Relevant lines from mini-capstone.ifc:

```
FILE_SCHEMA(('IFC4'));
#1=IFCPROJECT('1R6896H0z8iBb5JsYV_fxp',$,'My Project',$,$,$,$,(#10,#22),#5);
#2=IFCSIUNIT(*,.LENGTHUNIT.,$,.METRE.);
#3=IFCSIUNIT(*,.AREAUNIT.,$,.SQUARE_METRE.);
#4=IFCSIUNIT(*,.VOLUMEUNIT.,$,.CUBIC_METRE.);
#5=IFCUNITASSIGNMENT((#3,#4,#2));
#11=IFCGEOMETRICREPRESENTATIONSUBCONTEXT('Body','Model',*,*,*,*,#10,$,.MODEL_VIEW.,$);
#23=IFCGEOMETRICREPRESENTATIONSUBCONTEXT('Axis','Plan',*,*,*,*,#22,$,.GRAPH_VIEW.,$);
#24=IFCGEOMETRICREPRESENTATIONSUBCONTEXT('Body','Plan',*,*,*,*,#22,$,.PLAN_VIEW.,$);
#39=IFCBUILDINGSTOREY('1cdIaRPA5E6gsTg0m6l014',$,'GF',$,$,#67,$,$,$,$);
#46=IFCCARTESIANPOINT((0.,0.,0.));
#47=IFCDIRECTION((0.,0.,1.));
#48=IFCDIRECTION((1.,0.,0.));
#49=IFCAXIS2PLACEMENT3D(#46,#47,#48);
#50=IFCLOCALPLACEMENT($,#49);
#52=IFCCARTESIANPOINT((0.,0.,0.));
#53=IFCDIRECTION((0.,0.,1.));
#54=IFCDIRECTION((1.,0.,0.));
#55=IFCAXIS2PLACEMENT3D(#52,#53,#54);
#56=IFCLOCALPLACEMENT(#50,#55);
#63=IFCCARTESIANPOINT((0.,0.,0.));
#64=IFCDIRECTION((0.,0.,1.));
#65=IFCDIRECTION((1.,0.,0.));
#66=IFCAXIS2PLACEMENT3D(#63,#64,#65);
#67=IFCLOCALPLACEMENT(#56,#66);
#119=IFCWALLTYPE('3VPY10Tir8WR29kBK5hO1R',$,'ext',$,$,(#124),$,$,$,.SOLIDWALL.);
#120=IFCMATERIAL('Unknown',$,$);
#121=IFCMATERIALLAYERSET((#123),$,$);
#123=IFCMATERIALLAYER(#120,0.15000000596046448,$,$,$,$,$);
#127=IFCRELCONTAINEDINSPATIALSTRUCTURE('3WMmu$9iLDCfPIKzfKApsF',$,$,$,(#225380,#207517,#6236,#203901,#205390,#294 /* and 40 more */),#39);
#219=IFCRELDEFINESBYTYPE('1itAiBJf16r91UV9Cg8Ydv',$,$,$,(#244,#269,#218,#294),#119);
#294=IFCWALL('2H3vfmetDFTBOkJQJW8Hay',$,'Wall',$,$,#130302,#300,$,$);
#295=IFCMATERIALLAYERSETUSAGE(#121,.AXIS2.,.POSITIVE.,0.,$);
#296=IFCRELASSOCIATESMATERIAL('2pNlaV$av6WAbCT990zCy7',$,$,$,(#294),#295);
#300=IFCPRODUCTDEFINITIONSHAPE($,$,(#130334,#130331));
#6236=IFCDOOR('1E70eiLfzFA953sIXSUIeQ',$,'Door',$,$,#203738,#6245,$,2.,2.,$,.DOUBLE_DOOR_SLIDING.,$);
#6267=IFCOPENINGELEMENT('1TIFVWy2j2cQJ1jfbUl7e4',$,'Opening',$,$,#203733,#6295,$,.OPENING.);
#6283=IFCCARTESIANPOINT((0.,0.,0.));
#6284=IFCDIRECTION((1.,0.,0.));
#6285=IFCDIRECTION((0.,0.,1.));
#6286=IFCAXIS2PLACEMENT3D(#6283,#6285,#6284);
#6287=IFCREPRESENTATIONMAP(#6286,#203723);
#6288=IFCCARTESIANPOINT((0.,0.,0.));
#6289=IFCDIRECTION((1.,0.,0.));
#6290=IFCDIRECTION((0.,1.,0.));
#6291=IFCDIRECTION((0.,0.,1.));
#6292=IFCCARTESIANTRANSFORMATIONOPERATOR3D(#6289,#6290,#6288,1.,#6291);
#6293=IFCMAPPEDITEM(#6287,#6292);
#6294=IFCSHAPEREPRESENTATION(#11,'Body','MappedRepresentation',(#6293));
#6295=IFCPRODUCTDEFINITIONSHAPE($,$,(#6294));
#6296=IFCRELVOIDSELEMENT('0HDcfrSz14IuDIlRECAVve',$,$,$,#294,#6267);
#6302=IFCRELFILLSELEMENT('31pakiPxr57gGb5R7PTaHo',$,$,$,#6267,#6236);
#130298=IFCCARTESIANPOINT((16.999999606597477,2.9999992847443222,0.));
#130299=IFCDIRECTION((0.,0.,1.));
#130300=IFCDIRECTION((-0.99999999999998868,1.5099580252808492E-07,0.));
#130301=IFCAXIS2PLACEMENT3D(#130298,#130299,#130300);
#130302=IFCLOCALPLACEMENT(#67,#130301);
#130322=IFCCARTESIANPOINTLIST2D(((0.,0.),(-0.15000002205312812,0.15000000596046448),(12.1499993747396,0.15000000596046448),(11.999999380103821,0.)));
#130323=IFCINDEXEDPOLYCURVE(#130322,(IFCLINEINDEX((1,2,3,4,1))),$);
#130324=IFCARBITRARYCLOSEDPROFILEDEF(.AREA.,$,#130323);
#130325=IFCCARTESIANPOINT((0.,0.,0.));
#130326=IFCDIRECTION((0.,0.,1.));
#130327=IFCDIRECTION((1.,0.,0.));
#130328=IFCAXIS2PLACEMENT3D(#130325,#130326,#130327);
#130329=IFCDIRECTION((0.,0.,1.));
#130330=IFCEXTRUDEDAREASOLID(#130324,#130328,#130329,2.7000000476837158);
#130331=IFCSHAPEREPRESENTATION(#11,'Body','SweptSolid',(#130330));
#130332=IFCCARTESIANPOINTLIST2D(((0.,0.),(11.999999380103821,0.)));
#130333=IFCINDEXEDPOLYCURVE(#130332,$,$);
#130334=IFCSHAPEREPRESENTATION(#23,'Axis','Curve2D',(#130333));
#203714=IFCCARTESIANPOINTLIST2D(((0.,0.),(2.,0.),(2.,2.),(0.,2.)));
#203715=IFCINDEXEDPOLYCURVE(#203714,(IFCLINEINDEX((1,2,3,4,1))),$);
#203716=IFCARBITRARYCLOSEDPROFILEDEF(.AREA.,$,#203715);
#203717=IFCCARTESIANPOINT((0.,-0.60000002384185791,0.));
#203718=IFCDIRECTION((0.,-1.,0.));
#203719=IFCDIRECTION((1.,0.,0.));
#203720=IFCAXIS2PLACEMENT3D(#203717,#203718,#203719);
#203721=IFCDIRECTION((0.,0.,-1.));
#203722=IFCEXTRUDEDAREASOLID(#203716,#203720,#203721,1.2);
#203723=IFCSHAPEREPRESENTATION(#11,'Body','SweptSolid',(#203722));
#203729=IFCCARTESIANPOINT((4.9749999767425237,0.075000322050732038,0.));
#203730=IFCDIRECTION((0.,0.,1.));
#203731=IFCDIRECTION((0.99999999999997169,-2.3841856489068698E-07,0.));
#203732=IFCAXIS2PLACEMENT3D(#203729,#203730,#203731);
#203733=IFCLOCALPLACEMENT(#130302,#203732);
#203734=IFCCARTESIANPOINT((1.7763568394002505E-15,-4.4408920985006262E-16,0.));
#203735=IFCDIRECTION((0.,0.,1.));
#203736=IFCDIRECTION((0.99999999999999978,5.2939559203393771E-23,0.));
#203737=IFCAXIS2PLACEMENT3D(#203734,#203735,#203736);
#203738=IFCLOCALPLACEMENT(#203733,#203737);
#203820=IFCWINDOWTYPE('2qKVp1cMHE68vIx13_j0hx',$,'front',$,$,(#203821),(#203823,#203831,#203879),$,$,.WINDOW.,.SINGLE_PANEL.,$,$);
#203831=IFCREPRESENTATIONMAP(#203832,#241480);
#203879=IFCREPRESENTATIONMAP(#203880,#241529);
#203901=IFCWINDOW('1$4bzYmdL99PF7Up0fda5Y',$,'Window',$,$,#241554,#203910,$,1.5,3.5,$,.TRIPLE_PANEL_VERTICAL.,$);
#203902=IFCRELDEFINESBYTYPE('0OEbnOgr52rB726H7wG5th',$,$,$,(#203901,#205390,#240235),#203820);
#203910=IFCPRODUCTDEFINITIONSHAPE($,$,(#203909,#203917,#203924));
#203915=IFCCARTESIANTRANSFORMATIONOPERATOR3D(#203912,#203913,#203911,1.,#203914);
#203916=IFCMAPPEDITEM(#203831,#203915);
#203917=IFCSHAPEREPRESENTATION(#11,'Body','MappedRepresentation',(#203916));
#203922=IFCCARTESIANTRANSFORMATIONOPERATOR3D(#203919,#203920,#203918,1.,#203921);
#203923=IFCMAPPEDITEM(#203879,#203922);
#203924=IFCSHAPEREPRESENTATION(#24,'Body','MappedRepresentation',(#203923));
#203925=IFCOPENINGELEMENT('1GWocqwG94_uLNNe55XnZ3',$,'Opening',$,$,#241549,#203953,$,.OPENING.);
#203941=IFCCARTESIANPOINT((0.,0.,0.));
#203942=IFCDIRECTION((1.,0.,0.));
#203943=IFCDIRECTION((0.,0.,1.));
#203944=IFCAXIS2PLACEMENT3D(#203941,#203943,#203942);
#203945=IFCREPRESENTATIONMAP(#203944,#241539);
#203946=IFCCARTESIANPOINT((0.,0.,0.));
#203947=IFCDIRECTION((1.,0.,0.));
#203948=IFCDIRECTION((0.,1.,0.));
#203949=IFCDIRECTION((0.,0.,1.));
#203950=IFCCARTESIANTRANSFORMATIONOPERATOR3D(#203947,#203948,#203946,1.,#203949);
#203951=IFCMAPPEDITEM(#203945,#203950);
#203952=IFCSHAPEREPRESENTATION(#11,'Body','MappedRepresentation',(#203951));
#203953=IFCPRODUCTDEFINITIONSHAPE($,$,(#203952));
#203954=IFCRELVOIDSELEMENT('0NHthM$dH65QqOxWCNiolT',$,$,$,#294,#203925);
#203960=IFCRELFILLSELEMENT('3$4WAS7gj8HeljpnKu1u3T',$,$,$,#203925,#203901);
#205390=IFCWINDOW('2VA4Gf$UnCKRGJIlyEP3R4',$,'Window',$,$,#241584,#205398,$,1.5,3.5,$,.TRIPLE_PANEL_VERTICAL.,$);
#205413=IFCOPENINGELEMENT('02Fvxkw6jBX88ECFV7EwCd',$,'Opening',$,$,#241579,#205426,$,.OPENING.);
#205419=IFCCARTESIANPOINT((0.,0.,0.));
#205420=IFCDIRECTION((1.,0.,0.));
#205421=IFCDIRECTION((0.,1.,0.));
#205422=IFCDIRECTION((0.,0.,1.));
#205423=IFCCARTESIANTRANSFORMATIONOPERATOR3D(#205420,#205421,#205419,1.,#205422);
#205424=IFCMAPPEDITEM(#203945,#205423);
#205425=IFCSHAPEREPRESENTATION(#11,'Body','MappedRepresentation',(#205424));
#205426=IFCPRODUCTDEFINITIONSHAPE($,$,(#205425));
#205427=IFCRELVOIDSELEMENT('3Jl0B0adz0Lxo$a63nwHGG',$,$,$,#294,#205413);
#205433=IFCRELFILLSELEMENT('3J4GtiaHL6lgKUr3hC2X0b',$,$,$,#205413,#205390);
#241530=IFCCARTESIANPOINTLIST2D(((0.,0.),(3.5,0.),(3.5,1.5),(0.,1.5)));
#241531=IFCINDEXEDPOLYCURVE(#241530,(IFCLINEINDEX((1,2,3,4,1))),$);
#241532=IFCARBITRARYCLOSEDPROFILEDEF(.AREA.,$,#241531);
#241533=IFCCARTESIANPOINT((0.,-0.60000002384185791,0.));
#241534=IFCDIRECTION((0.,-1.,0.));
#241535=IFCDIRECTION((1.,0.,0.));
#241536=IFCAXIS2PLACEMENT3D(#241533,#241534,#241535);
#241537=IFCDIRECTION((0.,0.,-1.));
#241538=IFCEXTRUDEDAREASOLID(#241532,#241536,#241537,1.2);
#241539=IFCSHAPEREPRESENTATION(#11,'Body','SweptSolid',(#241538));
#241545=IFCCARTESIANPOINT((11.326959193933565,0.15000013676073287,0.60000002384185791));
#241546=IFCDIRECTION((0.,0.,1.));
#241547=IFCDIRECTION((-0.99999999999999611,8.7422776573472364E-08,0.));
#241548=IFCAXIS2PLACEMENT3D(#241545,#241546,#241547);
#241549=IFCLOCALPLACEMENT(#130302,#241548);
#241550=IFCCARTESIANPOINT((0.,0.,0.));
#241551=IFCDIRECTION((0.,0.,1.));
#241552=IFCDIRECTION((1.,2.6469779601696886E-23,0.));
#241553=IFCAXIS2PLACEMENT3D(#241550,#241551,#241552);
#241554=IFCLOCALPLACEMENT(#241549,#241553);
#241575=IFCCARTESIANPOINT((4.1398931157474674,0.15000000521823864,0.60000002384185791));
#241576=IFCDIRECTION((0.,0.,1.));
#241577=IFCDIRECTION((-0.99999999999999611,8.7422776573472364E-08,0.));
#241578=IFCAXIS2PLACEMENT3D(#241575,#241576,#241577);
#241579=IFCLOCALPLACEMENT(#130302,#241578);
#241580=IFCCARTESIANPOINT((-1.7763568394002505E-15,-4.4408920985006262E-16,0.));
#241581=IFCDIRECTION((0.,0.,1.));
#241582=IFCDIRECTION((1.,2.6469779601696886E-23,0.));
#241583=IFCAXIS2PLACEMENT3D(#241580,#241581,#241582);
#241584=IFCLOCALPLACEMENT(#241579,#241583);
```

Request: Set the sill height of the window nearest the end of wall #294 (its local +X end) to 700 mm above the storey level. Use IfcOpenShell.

```python
import numpy as np
import ifcopenshell
import ifcopenshell.api.geometry
import ifcopenshell.geom
import ifcopenshell.util.element
import ifcopenshell.util.placement
import ifcopenshell.util.shape
import ifcopenshell.util.unit

model = ifcopenshell.open("mini-capstone.ifc")
unit_scale = ifcopenshell.util.unit.calculate_unit_scale(model)

window = model.by_id(203901)
opening = window.FillsVoids[0].RelatingOpeningElement
storey = ifcopenshell.util.element.get_container(window, ifc_class="IfcBuildingStorey")
level = ifcopenshell.util.placement.get_local_placement(storey.ObjectPlacement)[2, 3]

# The opening's origin need not be at the sill, so measure its lowest point.
shape = ifcopenshell.geom.create_shape(ifcopenshell.geom.settings(), opening)
bottom = ifcopenshell.util.shape.get_shape_bottom_elevation(shape, shape.geometry) / unit_scale
dz = level + 0.7 - bottom

shift = np.array([0.0, 0.0, dz])
# The window is placed relative to its opening, so it follows when the opening moves.
matrix = ifcopenshell.util.placement.get_local_placement(opening.ObjectPlacement)
matrix[:3, 3] += shift
ifcopenshell.api.geometry.edit_object_placement(
    model, product=opening, matrix=matrix, is_si=False, should_transform_children=True
)

print(f"moved by {dz * unit_scale:+.3f} m")

model.write("mini-capstone_rev.ifc")
```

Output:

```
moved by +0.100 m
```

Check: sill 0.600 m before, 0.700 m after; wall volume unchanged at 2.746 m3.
